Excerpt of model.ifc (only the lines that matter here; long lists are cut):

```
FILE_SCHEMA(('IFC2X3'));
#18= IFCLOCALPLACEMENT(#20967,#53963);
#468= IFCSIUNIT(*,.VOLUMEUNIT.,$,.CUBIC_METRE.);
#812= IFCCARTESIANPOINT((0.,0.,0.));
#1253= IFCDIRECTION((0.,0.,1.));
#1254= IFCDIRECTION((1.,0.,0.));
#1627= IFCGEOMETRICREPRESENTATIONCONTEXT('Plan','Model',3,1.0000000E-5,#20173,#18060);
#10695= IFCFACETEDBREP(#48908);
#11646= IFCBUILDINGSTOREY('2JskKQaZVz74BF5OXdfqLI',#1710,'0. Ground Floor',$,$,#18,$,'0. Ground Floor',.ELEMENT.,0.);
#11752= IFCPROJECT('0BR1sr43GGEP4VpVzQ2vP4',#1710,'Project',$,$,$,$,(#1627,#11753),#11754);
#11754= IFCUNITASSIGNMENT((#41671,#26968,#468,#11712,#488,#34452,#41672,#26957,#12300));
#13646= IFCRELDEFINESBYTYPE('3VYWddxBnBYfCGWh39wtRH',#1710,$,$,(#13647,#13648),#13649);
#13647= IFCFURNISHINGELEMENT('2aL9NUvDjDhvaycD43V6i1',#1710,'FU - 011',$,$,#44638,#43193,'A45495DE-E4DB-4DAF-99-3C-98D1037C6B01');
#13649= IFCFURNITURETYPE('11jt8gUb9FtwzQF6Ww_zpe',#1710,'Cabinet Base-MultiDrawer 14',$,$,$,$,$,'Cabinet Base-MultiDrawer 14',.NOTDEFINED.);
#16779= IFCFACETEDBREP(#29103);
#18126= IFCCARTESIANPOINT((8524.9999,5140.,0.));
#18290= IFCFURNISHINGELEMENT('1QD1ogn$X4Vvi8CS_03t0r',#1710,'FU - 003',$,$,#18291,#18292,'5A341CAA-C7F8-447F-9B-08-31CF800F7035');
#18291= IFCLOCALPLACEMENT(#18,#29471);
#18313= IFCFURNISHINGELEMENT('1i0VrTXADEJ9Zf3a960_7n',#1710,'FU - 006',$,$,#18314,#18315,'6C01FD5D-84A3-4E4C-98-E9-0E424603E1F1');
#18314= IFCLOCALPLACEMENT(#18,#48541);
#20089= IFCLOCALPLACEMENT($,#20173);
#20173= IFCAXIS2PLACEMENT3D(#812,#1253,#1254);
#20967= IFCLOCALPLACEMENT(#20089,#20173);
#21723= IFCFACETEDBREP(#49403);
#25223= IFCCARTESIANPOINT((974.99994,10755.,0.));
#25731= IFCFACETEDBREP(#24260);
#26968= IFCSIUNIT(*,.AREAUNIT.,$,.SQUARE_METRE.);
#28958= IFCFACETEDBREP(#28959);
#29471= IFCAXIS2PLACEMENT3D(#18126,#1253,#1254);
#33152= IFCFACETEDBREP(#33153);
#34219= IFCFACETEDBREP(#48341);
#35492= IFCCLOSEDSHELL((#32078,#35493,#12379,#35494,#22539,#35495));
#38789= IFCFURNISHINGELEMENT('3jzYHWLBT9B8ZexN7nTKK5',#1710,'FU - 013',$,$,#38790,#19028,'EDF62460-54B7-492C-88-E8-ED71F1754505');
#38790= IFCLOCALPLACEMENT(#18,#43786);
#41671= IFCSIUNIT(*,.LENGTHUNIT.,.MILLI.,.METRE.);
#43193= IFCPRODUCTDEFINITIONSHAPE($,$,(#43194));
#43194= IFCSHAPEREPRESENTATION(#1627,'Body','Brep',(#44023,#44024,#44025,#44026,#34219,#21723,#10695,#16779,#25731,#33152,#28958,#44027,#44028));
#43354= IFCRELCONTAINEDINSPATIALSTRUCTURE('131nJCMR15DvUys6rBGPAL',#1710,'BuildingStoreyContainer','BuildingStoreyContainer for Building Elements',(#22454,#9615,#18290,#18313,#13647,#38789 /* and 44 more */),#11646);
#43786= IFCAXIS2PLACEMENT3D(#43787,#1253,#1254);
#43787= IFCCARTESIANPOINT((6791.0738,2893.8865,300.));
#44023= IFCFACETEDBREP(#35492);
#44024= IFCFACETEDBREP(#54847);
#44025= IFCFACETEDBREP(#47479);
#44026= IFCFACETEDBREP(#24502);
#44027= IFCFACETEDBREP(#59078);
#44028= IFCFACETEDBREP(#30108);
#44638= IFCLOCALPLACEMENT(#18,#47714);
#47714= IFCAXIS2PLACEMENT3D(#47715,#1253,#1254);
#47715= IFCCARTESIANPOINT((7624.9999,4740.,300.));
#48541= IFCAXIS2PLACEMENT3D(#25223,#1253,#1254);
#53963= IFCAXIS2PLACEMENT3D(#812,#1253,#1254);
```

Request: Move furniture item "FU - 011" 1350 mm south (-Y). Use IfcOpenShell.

```python
import ifcopenshell
import ifcopenshell.api.geometry
import ifcopenshell.util.placement
import ifcopenshell.util.unit

model = ifcopenshell.open("model.ifc")
unit_scale = ifcopenshell.util.unit.calculate_unit_scale(model)

item = model.by_guid("2aL9NUvDjDhvaycD43V6i1")
matrix = ifcopenshell.util.placement.get_local_placement(item.ObjectPlacement)
matrix[1, 3] -= 1.35 / unit_scale
ifcopenshell.api.geometry.edit_object_placement(model, product=item, matrix=matrix, is_si=False)

print(ifcopenshell.util.placement.get_local_placement(item.ObjectPlacement).round(3) + 0.0)

model.write("model_updated.ifc")
```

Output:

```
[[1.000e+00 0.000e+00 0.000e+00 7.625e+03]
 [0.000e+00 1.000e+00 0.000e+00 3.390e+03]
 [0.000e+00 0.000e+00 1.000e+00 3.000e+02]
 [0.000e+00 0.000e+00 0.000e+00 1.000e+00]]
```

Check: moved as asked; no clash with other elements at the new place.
